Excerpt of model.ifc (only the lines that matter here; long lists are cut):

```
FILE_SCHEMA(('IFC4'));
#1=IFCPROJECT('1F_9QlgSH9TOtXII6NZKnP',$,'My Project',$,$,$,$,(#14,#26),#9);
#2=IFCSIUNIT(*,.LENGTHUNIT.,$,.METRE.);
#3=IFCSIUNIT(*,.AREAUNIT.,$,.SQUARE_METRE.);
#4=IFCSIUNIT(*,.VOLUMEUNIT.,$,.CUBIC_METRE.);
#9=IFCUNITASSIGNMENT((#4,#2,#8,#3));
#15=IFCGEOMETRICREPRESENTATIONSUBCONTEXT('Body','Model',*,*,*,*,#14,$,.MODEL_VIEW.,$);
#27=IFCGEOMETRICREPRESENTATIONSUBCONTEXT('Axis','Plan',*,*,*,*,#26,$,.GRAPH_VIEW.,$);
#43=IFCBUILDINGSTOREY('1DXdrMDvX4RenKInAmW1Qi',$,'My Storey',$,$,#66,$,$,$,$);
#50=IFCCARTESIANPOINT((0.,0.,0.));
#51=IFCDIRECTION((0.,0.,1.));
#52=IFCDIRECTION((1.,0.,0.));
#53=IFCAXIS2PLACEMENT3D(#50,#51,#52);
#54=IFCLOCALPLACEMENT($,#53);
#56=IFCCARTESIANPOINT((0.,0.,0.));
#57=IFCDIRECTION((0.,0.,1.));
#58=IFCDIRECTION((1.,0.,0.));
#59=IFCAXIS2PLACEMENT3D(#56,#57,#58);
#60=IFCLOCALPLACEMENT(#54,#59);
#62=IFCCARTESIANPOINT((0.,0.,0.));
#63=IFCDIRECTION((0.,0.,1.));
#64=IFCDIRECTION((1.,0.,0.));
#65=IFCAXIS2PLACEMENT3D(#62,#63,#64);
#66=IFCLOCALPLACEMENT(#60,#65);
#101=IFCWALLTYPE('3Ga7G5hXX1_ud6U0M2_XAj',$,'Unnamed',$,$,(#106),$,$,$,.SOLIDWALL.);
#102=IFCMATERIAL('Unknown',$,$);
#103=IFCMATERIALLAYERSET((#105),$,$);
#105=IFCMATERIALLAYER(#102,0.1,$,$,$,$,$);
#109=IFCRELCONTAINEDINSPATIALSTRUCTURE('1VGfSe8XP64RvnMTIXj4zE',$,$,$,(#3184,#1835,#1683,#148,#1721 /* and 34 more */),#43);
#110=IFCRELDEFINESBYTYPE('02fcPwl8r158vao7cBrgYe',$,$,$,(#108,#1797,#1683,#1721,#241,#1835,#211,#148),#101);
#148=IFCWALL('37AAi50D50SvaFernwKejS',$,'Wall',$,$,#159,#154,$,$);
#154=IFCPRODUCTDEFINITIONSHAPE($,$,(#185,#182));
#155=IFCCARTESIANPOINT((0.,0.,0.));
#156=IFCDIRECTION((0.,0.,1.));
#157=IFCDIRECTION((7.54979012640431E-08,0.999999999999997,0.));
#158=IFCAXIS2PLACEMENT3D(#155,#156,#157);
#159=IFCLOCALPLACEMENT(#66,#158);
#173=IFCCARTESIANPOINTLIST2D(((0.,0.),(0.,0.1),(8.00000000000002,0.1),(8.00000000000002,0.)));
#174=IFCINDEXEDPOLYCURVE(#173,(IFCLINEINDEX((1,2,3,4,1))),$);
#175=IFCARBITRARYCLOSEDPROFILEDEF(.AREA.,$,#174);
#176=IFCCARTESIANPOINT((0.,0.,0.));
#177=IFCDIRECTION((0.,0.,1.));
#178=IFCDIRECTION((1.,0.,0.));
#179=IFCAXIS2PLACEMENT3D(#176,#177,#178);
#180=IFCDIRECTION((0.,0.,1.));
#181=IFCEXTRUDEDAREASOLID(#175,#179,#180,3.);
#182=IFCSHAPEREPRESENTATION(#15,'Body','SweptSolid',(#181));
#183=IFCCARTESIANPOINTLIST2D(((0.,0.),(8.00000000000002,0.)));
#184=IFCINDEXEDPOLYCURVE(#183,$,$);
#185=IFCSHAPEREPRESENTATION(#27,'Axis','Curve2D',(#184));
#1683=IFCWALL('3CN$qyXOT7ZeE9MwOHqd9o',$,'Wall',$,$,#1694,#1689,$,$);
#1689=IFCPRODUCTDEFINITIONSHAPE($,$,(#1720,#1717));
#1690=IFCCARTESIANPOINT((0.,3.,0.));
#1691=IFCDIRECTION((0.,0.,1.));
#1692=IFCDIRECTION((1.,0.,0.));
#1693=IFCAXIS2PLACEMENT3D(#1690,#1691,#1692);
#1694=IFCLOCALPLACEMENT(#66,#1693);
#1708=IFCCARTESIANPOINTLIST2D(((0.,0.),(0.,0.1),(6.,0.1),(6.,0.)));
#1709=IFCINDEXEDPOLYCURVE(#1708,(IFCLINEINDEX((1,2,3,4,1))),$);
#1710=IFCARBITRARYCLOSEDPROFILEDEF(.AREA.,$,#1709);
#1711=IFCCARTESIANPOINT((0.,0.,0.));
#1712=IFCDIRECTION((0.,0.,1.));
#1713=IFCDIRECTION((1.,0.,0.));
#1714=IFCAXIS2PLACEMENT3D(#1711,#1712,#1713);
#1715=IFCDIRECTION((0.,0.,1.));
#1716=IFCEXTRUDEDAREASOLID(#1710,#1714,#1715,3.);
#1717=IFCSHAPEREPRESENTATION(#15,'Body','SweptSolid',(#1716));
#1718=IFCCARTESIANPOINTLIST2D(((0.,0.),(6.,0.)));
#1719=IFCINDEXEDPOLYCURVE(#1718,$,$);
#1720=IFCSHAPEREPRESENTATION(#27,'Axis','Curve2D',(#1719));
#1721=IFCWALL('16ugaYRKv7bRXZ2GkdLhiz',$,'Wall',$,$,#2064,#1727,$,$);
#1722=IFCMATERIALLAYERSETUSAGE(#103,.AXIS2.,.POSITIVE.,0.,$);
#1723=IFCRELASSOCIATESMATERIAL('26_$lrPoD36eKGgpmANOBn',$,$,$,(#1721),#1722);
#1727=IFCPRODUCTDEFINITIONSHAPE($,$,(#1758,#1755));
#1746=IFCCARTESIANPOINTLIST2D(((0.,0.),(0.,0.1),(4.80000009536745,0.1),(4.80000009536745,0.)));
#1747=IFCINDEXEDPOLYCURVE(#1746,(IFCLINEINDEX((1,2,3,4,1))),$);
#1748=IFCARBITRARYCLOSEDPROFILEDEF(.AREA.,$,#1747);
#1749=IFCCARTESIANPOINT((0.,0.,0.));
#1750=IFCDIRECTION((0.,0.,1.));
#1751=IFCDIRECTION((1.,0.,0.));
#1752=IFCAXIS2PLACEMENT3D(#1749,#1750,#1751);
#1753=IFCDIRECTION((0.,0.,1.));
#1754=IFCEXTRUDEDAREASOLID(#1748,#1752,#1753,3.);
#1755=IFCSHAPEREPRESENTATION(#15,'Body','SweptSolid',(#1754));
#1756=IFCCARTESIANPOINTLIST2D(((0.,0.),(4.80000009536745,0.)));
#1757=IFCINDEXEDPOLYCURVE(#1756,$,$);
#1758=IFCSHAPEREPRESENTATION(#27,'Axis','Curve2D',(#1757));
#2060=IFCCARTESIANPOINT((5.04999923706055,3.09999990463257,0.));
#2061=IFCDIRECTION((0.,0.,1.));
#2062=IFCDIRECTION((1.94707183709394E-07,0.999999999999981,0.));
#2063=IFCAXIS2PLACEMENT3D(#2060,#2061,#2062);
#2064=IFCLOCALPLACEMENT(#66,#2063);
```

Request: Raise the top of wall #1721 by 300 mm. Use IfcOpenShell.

```python
import ifcopenshell
import ifcopenshell.geom
import ifcopenshell.util.representation
import ifcopenshell.util.shape

model = ifcopenshell.open("model.ifc")
settings = ifcopenshell.geom.settings()


def volume(element):
    """Net volume in cubic metres, openings subtracted."""
    shape = ifcopenshell.geom.create_shape(settings, element)
    return ifcopenshell.util.shape.get_volume(shape.geometry)


wall = model.by_id(1721)
before = volume(wall)

body = ifcopenshell.util.representation.get_representation(wall, "Model", "Body")
solid = body.Items[0]
old_height = solid.Depth
solid.Depth += 0.3
after = volume(wall)

print(f"height {old_height:g} -> {solid.Depth:g}, volume {before:.3f} -> {after:.3f} m3")

model.write("model_updated.ifc")
```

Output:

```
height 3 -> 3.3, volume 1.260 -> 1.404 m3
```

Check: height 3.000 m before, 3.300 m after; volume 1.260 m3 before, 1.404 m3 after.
